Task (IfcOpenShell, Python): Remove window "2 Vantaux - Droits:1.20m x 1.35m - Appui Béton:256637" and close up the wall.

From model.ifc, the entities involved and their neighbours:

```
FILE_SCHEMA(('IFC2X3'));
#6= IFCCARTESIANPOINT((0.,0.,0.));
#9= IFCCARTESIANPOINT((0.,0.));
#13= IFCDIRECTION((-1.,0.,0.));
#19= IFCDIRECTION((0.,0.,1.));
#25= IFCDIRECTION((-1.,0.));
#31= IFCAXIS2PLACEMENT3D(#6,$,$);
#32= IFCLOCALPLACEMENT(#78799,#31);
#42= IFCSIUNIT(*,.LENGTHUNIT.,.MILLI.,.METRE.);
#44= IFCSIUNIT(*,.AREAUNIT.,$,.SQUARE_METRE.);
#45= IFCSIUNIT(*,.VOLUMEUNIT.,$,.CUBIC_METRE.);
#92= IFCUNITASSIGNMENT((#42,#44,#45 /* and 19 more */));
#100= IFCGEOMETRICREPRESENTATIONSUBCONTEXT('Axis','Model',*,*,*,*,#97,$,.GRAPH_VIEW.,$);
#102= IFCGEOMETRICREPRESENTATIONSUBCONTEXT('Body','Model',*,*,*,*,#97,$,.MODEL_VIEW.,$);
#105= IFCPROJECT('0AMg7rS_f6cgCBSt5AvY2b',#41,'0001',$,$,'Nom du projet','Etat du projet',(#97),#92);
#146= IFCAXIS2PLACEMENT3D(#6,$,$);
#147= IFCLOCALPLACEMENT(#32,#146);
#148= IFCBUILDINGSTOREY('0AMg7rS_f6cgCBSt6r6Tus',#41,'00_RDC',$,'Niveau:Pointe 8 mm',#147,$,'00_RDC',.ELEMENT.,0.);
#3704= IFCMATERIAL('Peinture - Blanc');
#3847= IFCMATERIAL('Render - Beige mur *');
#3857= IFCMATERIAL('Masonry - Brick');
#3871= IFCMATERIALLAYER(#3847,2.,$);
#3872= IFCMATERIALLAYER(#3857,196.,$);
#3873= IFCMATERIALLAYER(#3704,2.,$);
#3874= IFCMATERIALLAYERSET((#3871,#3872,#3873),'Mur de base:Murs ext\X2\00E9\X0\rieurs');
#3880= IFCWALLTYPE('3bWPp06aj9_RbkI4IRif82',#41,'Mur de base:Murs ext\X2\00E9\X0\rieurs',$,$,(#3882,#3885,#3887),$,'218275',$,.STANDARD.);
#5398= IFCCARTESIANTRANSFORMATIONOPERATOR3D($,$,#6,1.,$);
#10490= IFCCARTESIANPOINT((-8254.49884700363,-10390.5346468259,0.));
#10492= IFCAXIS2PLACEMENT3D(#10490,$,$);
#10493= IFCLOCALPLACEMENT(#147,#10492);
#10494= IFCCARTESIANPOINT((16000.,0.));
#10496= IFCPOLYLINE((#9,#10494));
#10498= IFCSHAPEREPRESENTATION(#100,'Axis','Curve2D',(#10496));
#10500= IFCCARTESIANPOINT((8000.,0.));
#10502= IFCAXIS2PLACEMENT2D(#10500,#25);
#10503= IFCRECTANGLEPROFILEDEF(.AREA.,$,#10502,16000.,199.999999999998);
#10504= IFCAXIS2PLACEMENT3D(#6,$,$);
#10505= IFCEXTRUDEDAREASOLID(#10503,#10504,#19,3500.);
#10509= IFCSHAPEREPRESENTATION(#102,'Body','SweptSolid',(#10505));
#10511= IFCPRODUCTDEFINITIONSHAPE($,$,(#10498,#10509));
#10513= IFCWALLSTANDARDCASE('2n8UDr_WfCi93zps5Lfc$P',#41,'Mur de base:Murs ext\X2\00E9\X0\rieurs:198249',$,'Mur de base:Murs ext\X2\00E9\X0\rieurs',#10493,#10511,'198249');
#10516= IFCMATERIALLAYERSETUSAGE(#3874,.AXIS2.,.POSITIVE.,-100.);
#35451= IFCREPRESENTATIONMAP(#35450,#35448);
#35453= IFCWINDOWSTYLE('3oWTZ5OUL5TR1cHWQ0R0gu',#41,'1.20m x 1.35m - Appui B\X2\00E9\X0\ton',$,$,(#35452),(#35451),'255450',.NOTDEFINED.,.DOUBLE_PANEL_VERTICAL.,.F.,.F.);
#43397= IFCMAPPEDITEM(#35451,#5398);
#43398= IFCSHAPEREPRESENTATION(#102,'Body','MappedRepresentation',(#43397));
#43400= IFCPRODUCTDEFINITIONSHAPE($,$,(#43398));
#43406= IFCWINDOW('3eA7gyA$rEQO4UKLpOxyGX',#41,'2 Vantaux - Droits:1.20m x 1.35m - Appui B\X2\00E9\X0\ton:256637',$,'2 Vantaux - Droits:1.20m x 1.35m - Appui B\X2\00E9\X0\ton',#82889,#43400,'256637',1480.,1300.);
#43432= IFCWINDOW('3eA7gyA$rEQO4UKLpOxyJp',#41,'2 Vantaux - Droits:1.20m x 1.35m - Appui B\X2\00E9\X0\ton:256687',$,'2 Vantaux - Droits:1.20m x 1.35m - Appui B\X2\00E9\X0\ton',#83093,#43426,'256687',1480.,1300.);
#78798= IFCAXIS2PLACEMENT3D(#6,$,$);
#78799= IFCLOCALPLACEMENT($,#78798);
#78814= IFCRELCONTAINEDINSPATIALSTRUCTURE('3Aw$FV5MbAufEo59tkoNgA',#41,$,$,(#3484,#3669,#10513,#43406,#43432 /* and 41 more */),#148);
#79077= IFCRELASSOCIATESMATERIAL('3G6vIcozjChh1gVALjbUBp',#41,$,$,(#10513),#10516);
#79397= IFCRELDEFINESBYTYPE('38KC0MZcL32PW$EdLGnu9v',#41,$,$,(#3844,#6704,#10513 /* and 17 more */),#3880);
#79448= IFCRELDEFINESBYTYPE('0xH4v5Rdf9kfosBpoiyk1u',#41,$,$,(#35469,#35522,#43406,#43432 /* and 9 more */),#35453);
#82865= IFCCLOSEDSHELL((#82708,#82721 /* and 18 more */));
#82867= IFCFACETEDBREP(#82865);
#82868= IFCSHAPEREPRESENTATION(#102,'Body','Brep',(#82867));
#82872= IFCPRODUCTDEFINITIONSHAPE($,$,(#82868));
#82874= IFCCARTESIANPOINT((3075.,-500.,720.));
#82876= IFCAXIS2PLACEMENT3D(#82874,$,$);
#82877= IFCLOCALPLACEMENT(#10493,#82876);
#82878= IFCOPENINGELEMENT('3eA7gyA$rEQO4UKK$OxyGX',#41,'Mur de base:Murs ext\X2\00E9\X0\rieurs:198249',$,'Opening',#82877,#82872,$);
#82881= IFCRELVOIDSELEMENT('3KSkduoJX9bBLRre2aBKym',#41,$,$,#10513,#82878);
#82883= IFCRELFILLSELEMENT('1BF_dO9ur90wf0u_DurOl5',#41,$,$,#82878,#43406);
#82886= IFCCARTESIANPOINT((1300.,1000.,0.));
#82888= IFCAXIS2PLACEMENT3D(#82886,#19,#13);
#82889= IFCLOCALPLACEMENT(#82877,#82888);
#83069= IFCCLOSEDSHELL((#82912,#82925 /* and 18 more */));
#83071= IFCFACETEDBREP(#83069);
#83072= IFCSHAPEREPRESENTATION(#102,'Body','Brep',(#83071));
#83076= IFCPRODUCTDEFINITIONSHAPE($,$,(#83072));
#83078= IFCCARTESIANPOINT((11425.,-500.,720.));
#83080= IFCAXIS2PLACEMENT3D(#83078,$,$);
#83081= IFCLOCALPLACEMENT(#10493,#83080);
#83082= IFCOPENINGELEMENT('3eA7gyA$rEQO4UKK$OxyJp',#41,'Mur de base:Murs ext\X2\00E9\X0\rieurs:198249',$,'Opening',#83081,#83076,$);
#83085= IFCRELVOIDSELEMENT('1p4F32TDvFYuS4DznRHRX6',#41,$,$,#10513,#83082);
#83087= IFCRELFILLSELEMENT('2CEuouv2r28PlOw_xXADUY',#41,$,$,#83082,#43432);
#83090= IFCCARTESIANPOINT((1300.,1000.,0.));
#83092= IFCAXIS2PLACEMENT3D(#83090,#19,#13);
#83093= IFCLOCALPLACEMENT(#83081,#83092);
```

```python
import ifcopenshell
import ifcopenshell.api.feature
import ifcopenshell.api.root
import ifcopenshell.geom
import ifcopenshell.util.shape

model = ifcopenshell.open("model.ifc")
settings = ifcopenshell.geom.settings()


def volume(element):
    """Net volume in cubic metres, openings subtracted."""
    shape = ifcopenshell.geom.create_shape(settings, element)
    return ifcopenshell.util.shape.get_volume(shape.geometry)


window = model.by_guid("3eA7gyA$rEQO4UKLpOxyGX")
opening = window.FillsVoids[0].RelatingOpeningElement
wall = opening.VoidsElements[0].RelatingBuildingElement
before = volume(wall)

ifcopenshell.api.root.remove_product(model, product=window)
ifcopenshell.api.feature.remove_feature(model, feature=opening)

after = volume(wall)

print(f"wall volume {before:.3f} -> {after:.3f} m3")

model.write("model-out.ifc")
```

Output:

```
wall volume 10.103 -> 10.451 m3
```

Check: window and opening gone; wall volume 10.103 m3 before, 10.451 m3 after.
